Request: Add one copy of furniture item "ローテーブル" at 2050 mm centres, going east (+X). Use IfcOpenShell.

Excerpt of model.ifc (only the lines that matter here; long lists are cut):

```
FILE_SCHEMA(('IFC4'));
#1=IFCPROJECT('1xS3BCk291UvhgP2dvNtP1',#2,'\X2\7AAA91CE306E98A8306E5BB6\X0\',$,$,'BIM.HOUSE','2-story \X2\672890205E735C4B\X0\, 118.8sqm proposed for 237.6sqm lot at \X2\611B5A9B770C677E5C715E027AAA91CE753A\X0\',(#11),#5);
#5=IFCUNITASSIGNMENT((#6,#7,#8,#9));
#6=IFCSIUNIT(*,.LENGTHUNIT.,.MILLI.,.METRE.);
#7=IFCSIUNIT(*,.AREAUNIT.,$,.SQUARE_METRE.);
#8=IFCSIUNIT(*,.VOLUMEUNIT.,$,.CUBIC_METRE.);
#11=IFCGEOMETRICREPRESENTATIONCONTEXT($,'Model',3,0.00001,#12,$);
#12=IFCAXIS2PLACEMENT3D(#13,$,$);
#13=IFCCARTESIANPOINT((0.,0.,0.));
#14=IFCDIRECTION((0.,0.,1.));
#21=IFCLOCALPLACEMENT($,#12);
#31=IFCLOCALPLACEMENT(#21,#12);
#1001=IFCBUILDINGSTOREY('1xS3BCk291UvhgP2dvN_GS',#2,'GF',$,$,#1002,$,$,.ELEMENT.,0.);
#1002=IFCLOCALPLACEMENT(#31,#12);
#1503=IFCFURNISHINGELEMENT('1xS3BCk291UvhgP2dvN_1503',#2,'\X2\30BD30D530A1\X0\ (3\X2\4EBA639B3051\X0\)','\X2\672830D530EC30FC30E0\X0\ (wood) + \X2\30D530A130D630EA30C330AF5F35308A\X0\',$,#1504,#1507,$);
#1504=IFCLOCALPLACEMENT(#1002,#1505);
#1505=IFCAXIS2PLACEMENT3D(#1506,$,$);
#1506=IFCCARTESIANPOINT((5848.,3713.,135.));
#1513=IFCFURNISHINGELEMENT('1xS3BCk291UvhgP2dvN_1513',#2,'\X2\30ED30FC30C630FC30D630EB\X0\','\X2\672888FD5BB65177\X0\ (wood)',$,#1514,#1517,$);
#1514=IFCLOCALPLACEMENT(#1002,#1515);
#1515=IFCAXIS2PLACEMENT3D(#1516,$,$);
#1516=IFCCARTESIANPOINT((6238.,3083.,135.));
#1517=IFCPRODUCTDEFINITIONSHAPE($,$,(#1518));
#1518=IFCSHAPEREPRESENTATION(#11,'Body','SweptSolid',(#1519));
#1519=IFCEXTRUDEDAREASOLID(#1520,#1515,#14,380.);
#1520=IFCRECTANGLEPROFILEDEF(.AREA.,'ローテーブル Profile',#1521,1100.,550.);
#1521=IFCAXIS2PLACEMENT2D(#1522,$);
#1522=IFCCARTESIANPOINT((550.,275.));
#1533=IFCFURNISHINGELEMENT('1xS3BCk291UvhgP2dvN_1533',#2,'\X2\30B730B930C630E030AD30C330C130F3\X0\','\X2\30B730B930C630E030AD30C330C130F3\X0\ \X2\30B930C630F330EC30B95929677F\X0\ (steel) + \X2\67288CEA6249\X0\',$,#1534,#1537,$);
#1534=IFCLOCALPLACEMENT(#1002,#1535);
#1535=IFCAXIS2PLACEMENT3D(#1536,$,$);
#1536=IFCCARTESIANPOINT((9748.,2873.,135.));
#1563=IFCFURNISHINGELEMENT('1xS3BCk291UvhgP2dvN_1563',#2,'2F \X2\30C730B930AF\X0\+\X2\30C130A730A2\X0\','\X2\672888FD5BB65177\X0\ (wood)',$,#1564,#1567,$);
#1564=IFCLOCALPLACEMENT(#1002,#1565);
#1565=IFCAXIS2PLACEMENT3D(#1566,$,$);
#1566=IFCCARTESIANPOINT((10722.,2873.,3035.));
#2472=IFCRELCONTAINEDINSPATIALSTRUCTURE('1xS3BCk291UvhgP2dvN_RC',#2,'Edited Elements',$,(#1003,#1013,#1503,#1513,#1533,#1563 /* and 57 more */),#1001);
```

```python
import numpy as np
import ifcopenshell
import ifcopenshell.api.geometry
import ifcopenshell.api.root
import ifcopenshell.util.element
import ifcopenshell.util.placement
import ifcopenshell.util.unit

model = ifcopenshell.open("model.ifc")
unit_scale = ifcopenshell.util.unit.calculate_unit_scale(model)


def reuse_history(source, copy):
    """copy_class also copies each property set's owner history, people and application; keep the originals."""
    for rel in copy.IsDefinedBy:
        if rel.is_a("IfcRelDefinesByProperties") and (history := rel.RelatingPropertyDefinition.OwnerHistory):
            rel.RelatingPropertyDefinition.OwnerHistory = source.OwnerHistory
            ifcopenshell.util.element.remove_deep2(model, history)


source = model.by_id(1513)
base = ifcopenshell.util.placement.get_local_placement(source.ObjectPlacement)
step = np.array([1.0, 0.0, 0.0]) * 2.05 / unit_scale

for i in range(1, 2):
    copy = ifcopenshell.api.root.copy_class(model, product=source)
    copy.Representation = ifcopenshell.util.element.copy_deep(
        model, source.Representation, exclude=["IfcGeometricRepresentationContext", "IfcRepresentationMap"]
    )
    reuse_history(source, copy)
    matrix = base.copy()
    matrix[:3, 3] += i * step
    print("added at", matrix[:3, 3].round(3) + 0.0)
    ifcopenshell.api.geometry.edit_object_placement(model, product=copy, matrix=matrix, is_si=False)

model.write("model_v2.ifc")
```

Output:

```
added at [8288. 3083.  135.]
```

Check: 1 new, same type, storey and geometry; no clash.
